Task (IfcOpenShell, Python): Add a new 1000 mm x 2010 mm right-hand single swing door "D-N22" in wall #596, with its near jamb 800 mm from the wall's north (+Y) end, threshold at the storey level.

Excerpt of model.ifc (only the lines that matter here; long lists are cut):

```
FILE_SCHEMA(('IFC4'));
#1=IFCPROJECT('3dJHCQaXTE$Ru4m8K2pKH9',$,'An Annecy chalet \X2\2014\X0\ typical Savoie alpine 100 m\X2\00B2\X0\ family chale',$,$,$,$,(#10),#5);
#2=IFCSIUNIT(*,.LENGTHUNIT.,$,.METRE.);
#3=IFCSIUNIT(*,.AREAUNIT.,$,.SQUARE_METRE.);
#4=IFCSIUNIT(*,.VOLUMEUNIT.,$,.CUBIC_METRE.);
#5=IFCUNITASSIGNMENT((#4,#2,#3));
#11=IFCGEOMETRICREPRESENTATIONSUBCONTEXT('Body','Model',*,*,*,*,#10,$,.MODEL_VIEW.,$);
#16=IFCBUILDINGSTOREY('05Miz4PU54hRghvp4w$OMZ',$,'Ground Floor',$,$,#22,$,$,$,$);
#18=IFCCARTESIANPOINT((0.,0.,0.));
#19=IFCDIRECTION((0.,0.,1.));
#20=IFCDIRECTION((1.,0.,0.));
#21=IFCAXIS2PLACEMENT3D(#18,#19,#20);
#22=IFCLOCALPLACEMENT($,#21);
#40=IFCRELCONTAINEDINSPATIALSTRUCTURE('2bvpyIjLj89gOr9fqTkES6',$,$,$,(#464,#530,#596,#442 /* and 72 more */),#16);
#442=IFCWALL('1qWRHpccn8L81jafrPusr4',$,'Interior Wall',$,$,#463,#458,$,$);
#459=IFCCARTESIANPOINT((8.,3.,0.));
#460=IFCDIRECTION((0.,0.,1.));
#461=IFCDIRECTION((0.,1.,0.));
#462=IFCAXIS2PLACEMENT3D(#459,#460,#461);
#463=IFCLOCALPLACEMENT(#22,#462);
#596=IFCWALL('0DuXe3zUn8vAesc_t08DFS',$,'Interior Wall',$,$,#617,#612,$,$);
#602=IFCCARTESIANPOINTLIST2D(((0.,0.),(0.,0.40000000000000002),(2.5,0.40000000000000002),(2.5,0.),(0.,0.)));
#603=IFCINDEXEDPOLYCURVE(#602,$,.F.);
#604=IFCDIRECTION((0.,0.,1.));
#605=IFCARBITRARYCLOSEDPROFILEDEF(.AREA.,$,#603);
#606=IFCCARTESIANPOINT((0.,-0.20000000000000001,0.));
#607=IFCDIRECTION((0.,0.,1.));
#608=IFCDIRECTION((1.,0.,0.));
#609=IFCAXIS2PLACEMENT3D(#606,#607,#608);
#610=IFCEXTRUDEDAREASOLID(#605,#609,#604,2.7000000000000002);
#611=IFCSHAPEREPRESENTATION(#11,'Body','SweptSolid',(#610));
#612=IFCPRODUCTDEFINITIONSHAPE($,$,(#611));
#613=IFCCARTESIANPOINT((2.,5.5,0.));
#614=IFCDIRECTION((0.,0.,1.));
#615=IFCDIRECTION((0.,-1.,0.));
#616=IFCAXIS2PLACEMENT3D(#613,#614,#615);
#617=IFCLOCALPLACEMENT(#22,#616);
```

```python
import numpy as np
import ifcopenshell
import ifcopenshell.api.feature
import ifcopenshell.api.geometry
import ifcopenshell.api.root
import ifcopenshell.api.spatial
import ifcopenshell.geom
import ifcopenshell.util.element
import ifcopenshell.util.placement
import ifcopenshell.util.representation
import ifcopenshell.util.shape
import ifcopenshell.util.unit

model = ifcopenshell.open("model.ifc")
unit_scale = ifcopenshell.util.unit.calculate_unit_scale(model)
settings = ifcopenshell.geom.settings()


def volume(element):
    """Net volume in cubic metres, openings subtracted."""
    shape = ifcopenshell.geom.create_shape(settings, element)
    return ifcopenshell.util.shape.get_volume(shape.geometry)


wall = model.by_id(596)
storey = ifcopenshell.util.element.get_container(wall, ifc_class="IfcBuildingStorey")
context = ifcopenshell.util.representation.get_context(model, "Model", "Body", "MODEL_VIEW")
before = volume(wall)

width, height, from_end, sill = 1, 2.01, 0.8, 0.0  # metres

# The wall runs along its own X axis, and the end named is its -X end.
wall_shape = ifcopenshell.geom.create_shape(settings, wall)
x, y, z = ifcopenshell.util.shape.get_vertices(wall_shape.geometry).T
start = x.min() + from_end
face, thickness = float(y.min()), float(y.max() - y.min())
wall_matrix = ifcopenshell.util.placement.get_local_placement(wall.ObjectPlacement)
level = ifcopenshell.util.placement.get_local_placement(storey.ObjectPlacement)[2, 3]


def in_wall(x, y):
    """Placement at x, y metres in the wall's axes, at sill height."""
    matrix = wall_matrix.copy()
    matrix[:, 3] = wall_matrix @ np.array([x / unit_scale, y / unit_scale, 0.0, 1.0])
    matrix[2, 3] = level + sill / unit_scale
    return matrix


# Opening: a box that overshoots both wall faces by 50 mm.
opening = ifcopenshell.api.root.create_entity(model, ifc_class="IfcOpeningElement", predefined_type="OPENING")
box = ifcopenshell.api.geometry.add_wall_representation(
    model, context=context, length=width, height=height, thickness=thickness + 0.1
)
ifcopenshell.api.geometry.assign_representation(model, product=opening, representation=box)
ifcopenshell.api.geometry.edit_object_placement(model, product=opening, matrix=in_wall(start, face - 0.05), is_si=False)
ifcopenshell.api.feature.add_feature(model, feature=opening, element=wall)

door = ifcopenshell.api.root.create_entity(model, ifc_class="IfcDoor", name="D-N22", predefined_type="DOOR")
door.OverallWidth, door.OverallHeight = width / unit_scale, height / unit_scale
door.OperationType = "SINGLE_SWING_RIGHT"
body = ifcopenshell.api.geometry.add_door_representation(
    model,
    context=context,
    overall_width=door.OverallWidth,
    overall_height=door.OverallHeight,
    operation_type="SINGLE_SWING_RIGHT",
    lining_properties={"LiningDepth": thickness / unit_scale, "ThresholdDepth": thickness / unit_scale},
)
ifcopenshell.api.geometry.assign_representation(model, product=door, representation=body)
ifcopenshell.api.spatial.assign_container(model, products=[door], relating_structure=storey)
ifcopenshell.api.feature.add_filling(model, opening=opening, element=door)

# The lining spans the wall, so the door starts at the wall face.
ifcopenshell.api.geometry.edit_object_placement(model, product=door, matrix=in_wall(start, face), is_si=False)

after = volume(wall)

print(f"wall volume {before:.3f} -> {after:.3f} m3")

model.write("model_updated.ifc")
```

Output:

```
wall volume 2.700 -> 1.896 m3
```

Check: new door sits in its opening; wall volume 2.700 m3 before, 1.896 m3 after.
